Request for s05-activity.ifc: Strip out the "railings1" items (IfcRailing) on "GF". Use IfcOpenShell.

First a look at what the model holds.

```python
import ifcopenshell
import ifcopenshell.util.element

model = ifcopenshell.open("s05-activity.ifc")
print(model.schema)
storey = next(s for s in model.by_type("IfcBuildingStorey") if s.Name == "GF")
railings = [e for e in ifcopenshell.util.element.get_decomposition(storey) if e.is_a("IfcRailing")]
seen = {}
for e in railings:
    element_type = ifcopenshell.util.element.get_type(e)
    name = element_type.Name if element_type not in (None, e) else None
    seen[name] = seen.get(name, 0) + 1
for name, count in sorted(seen.items(), key=str):
    print(count, "x", name)
```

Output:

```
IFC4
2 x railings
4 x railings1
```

```python
import ifcopenshell
import ifcopenshell.api.root
import ifcopenshell.util.element

model = ifcopenshell.open("s05-activity.ifc")

storey = next(s for s in model.by_type("IfcBuildingStorey") if s.Name == "GF")
railings = [e for e in ifcopenshell.util.element.get_decomposition(storey) if e.is_a("IfcRailing")]
targets = [e for e in railings if (t := ifcopenshell.util.element.get_type(e)) not in (None, e) and t.Name == "railings1"]

for e in targets:
    ifcopenshell.api.root.remove_product(model, product=e)
print(len(targets), "removed")

model.write("s05-activity_rev.ifc")
```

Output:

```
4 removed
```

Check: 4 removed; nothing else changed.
